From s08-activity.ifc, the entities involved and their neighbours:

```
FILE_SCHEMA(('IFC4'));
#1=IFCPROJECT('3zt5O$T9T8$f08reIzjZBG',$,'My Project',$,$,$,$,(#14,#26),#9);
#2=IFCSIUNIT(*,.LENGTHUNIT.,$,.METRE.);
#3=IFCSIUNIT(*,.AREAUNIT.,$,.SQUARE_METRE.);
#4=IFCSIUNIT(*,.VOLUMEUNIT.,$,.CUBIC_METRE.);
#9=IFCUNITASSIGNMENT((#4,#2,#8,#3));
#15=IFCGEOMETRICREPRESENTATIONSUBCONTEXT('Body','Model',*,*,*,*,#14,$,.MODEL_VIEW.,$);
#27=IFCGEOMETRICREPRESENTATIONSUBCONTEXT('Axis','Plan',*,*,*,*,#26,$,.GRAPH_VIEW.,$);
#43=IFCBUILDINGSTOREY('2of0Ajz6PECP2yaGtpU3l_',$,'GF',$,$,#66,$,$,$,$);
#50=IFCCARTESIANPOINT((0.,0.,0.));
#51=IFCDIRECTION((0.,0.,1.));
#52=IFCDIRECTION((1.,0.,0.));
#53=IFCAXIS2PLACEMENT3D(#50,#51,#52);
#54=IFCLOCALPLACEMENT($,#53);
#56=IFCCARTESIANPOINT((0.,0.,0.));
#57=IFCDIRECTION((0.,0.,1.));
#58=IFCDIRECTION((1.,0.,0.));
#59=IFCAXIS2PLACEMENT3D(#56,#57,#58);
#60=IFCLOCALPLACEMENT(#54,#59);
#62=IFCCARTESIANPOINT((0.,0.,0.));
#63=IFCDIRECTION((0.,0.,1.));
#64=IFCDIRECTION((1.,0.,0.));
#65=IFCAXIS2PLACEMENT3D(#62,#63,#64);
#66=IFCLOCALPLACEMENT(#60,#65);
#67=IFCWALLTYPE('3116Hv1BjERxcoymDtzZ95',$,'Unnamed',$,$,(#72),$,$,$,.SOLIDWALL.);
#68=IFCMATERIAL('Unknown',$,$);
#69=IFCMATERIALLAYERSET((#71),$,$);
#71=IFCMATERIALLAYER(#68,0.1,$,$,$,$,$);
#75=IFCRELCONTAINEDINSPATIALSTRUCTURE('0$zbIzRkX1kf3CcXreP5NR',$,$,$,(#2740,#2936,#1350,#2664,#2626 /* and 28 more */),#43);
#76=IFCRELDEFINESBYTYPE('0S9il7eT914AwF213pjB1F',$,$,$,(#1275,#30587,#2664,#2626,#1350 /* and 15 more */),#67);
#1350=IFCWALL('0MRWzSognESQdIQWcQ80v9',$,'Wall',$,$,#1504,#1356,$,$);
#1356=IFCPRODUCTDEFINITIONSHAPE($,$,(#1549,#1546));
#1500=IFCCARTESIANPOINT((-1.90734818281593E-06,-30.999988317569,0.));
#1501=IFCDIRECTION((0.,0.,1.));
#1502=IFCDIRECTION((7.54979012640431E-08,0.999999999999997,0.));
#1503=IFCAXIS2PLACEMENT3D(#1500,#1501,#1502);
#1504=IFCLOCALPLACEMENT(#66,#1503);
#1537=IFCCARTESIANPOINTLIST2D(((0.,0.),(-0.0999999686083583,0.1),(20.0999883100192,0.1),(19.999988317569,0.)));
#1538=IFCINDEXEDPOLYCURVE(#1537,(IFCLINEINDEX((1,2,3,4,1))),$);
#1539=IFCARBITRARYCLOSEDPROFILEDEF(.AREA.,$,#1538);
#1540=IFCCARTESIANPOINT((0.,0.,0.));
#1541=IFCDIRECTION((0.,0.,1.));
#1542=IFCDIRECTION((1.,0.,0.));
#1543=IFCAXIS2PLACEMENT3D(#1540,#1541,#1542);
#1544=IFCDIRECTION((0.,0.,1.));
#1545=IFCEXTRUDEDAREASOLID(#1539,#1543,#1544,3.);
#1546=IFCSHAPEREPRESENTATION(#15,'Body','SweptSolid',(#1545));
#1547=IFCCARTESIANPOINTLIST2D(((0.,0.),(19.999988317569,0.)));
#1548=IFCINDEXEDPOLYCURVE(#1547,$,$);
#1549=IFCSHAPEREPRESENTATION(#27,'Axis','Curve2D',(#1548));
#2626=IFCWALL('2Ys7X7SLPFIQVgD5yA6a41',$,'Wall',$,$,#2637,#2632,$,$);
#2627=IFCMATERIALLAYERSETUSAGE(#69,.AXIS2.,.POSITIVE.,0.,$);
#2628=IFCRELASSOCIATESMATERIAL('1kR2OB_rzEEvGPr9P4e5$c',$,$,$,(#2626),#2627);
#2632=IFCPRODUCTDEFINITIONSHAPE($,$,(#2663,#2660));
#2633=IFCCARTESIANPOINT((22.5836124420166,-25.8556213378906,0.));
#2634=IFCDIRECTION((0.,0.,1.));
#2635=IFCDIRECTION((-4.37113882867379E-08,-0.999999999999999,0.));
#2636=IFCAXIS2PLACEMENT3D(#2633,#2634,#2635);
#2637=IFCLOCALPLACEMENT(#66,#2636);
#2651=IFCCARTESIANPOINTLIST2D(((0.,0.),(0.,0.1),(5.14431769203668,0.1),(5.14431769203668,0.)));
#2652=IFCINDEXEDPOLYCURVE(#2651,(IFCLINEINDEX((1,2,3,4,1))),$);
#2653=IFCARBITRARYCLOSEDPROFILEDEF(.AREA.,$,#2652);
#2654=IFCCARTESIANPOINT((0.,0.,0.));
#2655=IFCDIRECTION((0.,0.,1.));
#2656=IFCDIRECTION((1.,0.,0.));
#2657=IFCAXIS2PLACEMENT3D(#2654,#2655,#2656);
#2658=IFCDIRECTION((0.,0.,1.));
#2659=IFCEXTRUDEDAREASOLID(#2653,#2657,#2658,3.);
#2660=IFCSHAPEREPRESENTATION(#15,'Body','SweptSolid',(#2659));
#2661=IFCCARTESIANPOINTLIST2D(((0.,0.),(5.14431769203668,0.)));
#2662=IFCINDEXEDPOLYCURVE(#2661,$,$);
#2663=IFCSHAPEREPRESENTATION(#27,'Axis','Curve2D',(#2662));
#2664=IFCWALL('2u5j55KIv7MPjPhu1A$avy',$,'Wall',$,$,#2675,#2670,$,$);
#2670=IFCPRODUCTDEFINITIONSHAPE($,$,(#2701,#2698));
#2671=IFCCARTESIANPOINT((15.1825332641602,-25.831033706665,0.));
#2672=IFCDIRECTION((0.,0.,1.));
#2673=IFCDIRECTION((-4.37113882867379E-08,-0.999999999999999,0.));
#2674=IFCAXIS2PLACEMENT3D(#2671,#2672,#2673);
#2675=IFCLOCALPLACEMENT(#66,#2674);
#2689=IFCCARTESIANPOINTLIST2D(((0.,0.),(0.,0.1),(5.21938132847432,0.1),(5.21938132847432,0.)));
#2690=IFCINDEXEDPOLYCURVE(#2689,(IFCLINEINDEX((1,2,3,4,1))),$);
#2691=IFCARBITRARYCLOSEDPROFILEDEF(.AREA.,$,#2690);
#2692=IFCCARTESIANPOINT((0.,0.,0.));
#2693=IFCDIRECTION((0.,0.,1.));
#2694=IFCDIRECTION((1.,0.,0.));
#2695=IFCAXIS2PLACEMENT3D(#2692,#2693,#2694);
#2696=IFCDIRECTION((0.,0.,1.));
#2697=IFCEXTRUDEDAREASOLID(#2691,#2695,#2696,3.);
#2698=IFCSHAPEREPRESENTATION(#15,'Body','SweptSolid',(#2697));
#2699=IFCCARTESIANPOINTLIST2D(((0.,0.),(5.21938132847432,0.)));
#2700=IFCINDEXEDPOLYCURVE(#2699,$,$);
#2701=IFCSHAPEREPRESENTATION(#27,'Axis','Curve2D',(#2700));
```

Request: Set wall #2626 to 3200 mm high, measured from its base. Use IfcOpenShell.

```python
import ifcopenshell
import ifcopenshell.geom
import ifcopenshell.util.representation
import ifcopenshell.util.shape

model = ifcopenshell.open("s08-activity.ifc")
settings = ifcopenshell.geom.settings()


def volume(element):
    """Net volume in cubic metres, openings subtracted."""
    shape = ifcopenshell.geom.create_shape(settings, element)
    return ifcopenshell.util.shape.get_volume(shape.geometry)


wall = model.by_id(2626)
before = volume(wall)

body = ifcopenshell.util.representation.get_representation(wall, "Model", "Body")
solid = body.Items[0]
old_height = solid.Depth
solid.Depth = 3.2
after = volume(wall)

print(f"height {old_height:g} -> {solid.Depth:g}, volume {before:.3f} -> {after:.3f} m3")

model.write("s08-activity_edited.ifc")
```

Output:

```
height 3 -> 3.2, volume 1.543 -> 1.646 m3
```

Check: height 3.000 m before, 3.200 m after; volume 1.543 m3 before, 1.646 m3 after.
